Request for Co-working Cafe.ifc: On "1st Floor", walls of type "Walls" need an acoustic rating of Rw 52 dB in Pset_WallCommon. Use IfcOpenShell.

First a look at what the model holds.

```python
import ifcopenshell
import ifcopenshell.util.element

model = ifcopenshell.open("Co-working Cafe.ifc")
print(model.schema)
storey = next(s for s in model.by_type("IfcBuildingStorey") if s.Name == "1st Floor")
walls = [e for e in ifcopenshell.util.element.get_decomposition(storey) if e.is_a("IfcWall")]
seen = {}
for e in walls:
    element_type = ifcopenshell.util.element.get_type(e)
    key = (element_type.Name if element_type != e and element_type else None, ifcopenshell.util.element.get_pset(e, "Pset_WallCommon", "AcousticRating"))
    seen[key] = seen.get(key, 0) + 1
for (name, value), count in sorted(seen.items(), key=str):
    print(count, "x", name, "|", value)
```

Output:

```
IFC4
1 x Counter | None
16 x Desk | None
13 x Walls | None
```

```python
import ifcopenshell
import ifcopenshell.api.pset
import ifcopenshell.util.element

model = ifcopenshell.open("Co-working Cafe.ifc")

storey = next(s for s in model.by_type("IfcBuildingStorey") if s.Name == "1st Floor")
walls = [e for e in ifcopenshell.util.element.get_decomposition(storey) if e.is_a("IfcWall")]

count = 0
for e in walls:
    element_type = ifcopenshell.util.element.get_type(e)
    if element_type in (None, e) or element_type.Name != "Walls":
        continue
    # add_pset returns the element's existing set when there is one.
    pset = ifcopenshell.api.pset.add_pset(model, product=e, name="Pset_WallCommon")
    ifcopenshell.api.pset.edit_pset(model, pset=pset, properties={"AcousticRating": "Rw 52 dB"})
    count += 1

print(count, "walls updated")

model.write("Co-working Cafe_edited.ifc")
```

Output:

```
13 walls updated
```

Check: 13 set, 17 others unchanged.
